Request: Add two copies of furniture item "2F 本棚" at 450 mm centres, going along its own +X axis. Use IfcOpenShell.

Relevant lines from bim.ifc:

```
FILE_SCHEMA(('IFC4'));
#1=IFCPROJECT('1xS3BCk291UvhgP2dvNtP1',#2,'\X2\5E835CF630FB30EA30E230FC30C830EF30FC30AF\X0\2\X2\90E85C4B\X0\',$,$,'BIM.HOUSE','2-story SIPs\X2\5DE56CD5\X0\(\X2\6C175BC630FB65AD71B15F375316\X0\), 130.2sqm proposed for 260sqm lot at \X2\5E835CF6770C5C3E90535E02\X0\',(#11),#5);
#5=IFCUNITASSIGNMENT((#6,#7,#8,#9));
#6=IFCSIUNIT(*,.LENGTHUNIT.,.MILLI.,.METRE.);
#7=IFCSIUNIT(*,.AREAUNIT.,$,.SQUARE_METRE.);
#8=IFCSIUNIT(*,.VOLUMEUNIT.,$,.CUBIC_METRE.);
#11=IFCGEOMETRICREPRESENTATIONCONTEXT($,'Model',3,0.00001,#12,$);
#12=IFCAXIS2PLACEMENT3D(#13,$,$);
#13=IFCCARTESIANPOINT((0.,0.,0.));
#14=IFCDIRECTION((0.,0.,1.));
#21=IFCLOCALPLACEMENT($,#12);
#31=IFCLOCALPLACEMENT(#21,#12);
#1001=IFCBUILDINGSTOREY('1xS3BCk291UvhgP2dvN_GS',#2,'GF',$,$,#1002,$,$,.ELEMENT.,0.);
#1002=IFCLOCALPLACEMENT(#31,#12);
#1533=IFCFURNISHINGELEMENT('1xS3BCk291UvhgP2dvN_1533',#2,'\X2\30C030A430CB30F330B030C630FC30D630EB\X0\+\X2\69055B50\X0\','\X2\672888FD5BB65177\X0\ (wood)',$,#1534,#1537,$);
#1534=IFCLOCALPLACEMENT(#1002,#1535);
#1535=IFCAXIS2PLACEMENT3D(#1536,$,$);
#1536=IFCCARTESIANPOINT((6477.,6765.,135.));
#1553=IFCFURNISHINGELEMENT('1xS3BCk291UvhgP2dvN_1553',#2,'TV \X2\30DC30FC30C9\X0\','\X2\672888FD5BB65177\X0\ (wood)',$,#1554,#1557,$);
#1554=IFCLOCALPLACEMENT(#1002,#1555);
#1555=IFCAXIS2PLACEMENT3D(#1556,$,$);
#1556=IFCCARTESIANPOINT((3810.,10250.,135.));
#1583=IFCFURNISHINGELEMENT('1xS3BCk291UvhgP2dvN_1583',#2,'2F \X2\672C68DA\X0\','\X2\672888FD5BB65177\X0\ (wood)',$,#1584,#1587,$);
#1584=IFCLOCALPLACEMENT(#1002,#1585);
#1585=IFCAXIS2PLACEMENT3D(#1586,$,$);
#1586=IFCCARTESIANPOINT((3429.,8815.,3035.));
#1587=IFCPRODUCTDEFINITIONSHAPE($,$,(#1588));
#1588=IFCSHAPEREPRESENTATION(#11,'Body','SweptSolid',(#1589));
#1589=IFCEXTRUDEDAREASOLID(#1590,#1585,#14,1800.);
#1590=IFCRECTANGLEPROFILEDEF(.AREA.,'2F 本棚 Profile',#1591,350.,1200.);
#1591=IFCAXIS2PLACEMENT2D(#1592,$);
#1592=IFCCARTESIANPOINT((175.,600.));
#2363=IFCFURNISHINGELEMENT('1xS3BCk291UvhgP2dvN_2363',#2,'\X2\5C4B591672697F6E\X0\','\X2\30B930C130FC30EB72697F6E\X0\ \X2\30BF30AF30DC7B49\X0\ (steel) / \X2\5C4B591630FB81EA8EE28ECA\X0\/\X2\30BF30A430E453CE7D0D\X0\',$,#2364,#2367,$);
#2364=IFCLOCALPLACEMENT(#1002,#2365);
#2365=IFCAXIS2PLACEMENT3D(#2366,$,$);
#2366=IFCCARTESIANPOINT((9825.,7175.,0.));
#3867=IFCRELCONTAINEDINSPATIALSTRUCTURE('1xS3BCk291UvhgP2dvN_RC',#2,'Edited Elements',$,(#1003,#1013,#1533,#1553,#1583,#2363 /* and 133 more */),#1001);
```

```python
import ifcopenshell
import ifcopenshell.api.geometry
import ifcopenshell.api.root
import ifcopenshell.util.element
import ifcopenshell.util.placement

model = ifcopenshell.open("bim.ifc")


def reuse_history(source, copy):
    """copy_class also copies each property set's owner history, people and application; keep the originals."""
    for rel in copy.IsDefinedBy:
        if rel.is_a("IfcRelDefinesByProperties") and (history := rel.RelatingPropertyDefinition.OwnerHistory):
            rel.RelatingPropertyDefinition.OwnerHistory = source.OwnerHistory
            ifcopenshell.util.element.remove_deep2(model, history)


source = model.by_guid("1xS3BCk291UvhgP2dvN_1583")
base = ifcopenshell.util.placement.get_local_placement(source.ObjectPlacement)
step = base[:3, 0] * 450.0

for i in range(1, 3):
    copy = ifcopenshell.api.root.copy_class(model, product=source)
    copy.Representation = ifcopenshell.util.element.copy_deep(
        model, source.Representation, exclude=["IfcGeometricRepresentationContext", "IfcRepresentationMap"]
    )
    reuse_history(source, copy)
    matrix = base.copy()
    matrix[:3, 3] += i * step
    print("added at", matrix[:3, 3].round(3) + 0.0)
    ifcopenshell.api.geometry.edit_object_placement(model, product=copy, matrix=matrix, is_si=False)

model.write("bim_edited.ifc")
```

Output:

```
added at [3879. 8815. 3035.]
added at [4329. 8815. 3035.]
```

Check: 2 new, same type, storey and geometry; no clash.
